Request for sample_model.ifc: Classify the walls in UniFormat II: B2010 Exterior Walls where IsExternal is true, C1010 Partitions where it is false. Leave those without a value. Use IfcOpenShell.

First a look at what the model holds.

```python
import ifcopenshell
import ifcopenshell.util.element

model = ifcopenshell.open("sample_model.ifc")
print(model.schema)
print("classifications:", [c.Name for c in model.by_type("IfcClassification")])
values = [ifcopenshell.util.element.get_pset(e, "Pset_WallCommon", "IsExternal") for e in model.by_type("IfcWall")]
for value in (True, False, None):
    print("IsExternal", value, values.count(value))
```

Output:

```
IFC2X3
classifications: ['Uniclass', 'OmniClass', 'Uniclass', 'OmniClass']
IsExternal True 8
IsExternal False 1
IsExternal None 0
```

```python
import ifcopenshell
import ifcopenshell.api.classification
import ifcopenshell.util.element

model = ifcopenshell.open("sample_model.ifc")

# IFC2X3 requires Source and Edition and has no link from the project to the system.
system = model.create_entity("IfcClassification", Source="ASTM", Edition="E1557", Name="UniFormat II")

walls = model.by_type("IfcWall")
external = {e: ifcopenshell.util.element.get_pset(e, "Pset_WallCommon", "IsExternal") for e in walls}
for flag, code, name in ((True, "B2010", "Exterior Walls"), (False, "C1010", "Partitions")):
    products = [e for e in walls if external[e] is flag]
    ifcopenshell.api.classification.add_reference(
        model, products=products, classification=system, identification=code, name=name
    )
    print(code, len(products))

model.write("sample_model_v2.ifc")
```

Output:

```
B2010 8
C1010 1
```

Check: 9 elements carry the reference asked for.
